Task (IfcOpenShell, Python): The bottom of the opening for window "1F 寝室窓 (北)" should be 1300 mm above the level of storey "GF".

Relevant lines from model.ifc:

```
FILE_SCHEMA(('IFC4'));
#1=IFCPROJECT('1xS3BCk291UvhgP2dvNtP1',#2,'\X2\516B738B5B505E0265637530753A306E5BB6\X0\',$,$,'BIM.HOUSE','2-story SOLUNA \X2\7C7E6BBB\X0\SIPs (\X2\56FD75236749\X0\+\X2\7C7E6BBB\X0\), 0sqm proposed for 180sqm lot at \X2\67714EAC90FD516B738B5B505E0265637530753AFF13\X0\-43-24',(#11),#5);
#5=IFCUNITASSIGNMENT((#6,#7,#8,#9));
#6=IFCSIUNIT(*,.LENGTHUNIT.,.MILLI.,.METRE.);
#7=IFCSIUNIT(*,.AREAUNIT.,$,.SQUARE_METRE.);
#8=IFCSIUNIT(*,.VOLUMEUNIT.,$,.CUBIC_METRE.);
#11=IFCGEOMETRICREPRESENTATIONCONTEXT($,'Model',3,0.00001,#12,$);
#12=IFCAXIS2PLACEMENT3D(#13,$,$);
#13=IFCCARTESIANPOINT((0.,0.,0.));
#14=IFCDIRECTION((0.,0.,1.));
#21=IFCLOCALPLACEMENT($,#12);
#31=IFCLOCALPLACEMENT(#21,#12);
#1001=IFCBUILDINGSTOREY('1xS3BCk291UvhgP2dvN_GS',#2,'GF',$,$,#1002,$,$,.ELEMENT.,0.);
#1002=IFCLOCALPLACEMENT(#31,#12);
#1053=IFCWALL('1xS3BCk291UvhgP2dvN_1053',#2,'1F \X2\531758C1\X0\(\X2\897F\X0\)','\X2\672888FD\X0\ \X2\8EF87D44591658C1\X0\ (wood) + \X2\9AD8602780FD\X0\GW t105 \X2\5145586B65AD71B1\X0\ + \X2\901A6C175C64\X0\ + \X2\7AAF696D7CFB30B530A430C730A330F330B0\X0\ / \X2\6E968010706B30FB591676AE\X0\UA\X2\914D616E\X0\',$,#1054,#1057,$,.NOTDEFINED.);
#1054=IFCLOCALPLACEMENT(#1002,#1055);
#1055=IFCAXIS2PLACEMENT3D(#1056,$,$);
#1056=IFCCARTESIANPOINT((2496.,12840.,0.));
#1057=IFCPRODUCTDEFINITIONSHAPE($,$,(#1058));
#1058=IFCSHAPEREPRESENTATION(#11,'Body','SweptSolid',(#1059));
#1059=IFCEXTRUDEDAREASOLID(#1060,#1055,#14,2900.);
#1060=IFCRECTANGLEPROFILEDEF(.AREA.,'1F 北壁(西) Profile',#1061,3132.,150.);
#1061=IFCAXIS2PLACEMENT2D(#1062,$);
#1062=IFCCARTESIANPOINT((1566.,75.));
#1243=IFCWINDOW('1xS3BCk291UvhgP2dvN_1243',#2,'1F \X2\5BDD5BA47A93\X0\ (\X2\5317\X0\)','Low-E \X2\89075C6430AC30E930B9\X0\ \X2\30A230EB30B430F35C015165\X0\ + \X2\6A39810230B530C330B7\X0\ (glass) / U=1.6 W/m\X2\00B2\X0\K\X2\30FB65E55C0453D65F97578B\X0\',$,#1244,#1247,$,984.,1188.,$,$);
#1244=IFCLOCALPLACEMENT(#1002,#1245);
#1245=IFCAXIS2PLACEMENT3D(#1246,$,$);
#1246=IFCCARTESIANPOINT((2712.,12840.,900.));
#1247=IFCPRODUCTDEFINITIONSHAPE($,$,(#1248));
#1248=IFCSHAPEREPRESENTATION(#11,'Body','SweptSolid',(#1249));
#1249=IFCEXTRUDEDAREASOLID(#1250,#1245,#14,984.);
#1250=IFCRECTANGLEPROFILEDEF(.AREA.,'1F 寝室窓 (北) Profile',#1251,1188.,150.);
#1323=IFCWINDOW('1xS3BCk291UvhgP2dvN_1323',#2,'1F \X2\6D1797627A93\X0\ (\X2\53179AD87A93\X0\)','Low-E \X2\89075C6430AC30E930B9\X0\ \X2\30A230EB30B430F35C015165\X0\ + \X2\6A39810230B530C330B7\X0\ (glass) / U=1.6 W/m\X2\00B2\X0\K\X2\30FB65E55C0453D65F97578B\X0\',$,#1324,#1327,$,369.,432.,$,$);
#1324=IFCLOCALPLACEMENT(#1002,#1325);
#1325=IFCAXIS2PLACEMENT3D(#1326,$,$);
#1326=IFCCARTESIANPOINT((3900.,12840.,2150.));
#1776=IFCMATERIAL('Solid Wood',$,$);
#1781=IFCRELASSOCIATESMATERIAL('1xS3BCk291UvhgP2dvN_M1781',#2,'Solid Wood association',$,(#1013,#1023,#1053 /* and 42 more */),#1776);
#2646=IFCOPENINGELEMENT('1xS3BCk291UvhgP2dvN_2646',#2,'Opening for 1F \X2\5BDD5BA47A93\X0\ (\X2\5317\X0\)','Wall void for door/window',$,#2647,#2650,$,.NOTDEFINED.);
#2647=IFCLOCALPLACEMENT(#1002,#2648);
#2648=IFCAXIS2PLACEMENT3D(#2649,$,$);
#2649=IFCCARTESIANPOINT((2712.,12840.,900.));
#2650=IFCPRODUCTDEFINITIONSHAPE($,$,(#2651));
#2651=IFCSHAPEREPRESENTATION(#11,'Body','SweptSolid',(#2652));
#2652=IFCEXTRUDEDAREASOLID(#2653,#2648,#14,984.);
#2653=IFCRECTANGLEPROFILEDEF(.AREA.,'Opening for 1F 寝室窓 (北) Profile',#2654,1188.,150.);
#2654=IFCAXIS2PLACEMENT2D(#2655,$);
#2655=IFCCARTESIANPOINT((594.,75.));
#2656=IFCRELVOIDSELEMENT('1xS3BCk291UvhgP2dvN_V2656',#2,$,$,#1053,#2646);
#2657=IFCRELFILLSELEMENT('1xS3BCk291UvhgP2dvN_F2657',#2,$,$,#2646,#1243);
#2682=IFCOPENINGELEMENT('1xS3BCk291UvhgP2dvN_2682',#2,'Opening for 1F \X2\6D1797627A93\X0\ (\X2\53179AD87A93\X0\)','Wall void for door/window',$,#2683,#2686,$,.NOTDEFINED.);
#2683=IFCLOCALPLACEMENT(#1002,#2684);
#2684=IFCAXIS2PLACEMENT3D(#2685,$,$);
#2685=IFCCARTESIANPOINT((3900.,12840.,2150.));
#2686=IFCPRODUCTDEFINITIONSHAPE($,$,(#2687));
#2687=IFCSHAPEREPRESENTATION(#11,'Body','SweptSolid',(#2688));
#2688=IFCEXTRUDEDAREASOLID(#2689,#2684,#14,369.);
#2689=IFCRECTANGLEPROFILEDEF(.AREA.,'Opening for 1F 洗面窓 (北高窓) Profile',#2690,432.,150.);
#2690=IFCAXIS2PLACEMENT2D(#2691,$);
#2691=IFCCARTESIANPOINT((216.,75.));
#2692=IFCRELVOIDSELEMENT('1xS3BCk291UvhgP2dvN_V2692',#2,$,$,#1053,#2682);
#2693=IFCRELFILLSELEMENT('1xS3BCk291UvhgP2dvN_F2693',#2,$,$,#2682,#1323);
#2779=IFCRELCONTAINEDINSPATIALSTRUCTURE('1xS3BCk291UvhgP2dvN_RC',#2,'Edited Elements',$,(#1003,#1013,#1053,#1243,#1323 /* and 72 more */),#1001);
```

```python
import numpy as np
import ifcopenshell
import ifcopenshell.api.geometry
import ifcopenshell.geom
import ifcopenshell.util.element
import ifcopenshell.util.placement
import ifcopenshell.util.shape
import ifcopenshell.util.unit

model = ifcopenshell.open("model.ifc")
unit_scale = ifcopenshell.util.unit.calculate_unit_scale(model)

window = model.by_guid("1xS3BCk291UvhgP2dvN_1243")
opening = window.FillsVoids[0].RelatingOpeningElement
storey = ifcopenshell.util.element.get_container(window, ifc_class="IfcBuildingStorey")
level = ifcopenshell.util.placement.get_local_placement(storey.ObjectPlacement)[2, 3]

# The opening's origin need not be at the sill, so measure its lowest point.
shape = ifcopenshell.geom.create_shape(ifcopenshell.geom.settings(), opening)
bottom = ifcopenshell.util.shape.get_shape_bottom_elevation(shape, shape.geometry) / unit_scale
dz = level + 1300.0 - bottom

shift = np.array([0.0, 0.0, dz])
# The window is not placed relative to its opening, so move both.
for product in (opening, window):
    matrix = ifcopenshell.util.placement.get_local_placement(product.ObjectPlacement)
    matrix[:3, 3] += shift
    ifcopenshell.api.geometry.edit_object_placement(model, product=product, matrix=matrix, is_si=False)

print(f"moved by {dz * unit_scale:+.3f} m")

model.write("model_updated.ifc")
```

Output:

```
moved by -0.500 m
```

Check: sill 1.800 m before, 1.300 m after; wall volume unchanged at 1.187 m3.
